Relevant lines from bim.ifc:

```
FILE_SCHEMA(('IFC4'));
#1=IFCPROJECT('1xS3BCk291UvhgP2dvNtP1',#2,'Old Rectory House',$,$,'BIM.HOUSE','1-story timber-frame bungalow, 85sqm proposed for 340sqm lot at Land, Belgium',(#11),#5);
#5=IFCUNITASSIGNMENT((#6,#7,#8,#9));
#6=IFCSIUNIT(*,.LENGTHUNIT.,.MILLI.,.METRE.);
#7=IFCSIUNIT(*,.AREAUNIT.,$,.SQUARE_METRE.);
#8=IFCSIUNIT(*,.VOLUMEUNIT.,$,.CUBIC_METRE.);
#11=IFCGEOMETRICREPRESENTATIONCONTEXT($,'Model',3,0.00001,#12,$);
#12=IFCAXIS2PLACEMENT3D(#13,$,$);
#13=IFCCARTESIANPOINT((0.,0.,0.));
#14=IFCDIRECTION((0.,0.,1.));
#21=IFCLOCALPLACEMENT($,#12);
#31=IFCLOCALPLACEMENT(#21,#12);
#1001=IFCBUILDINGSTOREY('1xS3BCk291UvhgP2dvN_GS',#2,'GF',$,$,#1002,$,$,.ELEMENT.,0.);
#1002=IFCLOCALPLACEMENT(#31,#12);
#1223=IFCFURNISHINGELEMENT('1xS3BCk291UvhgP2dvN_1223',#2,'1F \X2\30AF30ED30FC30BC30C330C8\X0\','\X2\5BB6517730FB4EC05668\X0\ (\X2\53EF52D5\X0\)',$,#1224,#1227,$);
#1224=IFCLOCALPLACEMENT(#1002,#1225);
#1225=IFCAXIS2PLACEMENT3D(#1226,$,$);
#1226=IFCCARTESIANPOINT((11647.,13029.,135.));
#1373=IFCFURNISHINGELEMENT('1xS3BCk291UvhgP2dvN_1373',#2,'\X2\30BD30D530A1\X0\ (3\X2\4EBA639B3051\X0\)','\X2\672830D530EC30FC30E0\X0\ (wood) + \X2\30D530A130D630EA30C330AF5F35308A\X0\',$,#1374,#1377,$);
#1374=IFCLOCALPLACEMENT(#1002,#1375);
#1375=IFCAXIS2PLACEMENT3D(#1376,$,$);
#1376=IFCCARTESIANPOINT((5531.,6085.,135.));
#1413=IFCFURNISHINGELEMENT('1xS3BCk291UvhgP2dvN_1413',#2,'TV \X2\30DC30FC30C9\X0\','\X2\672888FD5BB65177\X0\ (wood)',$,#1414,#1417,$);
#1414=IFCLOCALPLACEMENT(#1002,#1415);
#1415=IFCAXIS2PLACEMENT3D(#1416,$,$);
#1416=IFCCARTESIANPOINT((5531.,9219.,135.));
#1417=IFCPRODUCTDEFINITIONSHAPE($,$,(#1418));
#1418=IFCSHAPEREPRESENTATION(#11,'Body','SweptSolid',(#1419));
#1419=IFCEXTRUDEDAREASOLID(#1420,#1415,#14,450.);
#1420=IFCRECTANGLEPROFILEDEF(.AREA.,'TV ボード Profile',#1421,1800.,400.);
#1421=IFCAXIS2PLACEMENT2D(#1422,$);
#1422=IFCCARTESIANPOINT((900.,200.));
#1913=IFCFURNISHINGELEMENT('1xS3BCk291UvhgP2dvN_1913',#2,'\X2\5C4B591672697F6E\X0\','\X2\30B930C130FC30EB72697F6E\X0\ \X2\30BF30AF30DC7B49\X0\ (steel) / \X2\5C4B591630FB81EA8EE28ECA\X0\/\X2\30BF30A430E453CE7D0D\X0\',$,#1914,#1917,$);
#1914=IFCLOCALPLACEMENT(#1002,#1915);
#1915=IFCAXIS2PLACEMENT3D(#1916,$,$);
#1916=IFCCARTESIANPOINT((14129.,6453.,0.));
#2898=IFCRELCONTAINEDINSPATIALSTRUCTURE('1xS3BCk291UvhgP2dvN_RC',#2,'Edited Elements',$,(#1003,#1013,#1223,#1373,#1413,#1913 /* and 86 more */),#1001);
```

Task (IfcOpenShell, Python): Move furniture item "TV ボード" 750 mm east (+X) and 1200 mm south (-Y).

```python
import ifcopenshell
import ifcopenshell.api.geometry
import ifcopenshell.util.placement
import ifcopenshell.util.unit

model = ifcopenshell.open("bim.ifc")
unit_scale = ifcopenshell.util.unit.calculate_unit_scale(model)

item = model.by_id(1413)
matrix = ifcopenshell.util.placement.get_local_placement(item.ObjectPlacement)
matrix[0, 3] += 0.75 / unit_scale
matrix[1, 3] -= 1.2 / unit_scale
ifcopenshell.api.geometry.edit_object_placement(model, product=item, matrix=matrix, is_si=False)

print(ifcopenshell.util.placement.get_local_placement(item.ObjectPlacement).round(3) + 0.0)

model.write("bim_updated.ifc")
```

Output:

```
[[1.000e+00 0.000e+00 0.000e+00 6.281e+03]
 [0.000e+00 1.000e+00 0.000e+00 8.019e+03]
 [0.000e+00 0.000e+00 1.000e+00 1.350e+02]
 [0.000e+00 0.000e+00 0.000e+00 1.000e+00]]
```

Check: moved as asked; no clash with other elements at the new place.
